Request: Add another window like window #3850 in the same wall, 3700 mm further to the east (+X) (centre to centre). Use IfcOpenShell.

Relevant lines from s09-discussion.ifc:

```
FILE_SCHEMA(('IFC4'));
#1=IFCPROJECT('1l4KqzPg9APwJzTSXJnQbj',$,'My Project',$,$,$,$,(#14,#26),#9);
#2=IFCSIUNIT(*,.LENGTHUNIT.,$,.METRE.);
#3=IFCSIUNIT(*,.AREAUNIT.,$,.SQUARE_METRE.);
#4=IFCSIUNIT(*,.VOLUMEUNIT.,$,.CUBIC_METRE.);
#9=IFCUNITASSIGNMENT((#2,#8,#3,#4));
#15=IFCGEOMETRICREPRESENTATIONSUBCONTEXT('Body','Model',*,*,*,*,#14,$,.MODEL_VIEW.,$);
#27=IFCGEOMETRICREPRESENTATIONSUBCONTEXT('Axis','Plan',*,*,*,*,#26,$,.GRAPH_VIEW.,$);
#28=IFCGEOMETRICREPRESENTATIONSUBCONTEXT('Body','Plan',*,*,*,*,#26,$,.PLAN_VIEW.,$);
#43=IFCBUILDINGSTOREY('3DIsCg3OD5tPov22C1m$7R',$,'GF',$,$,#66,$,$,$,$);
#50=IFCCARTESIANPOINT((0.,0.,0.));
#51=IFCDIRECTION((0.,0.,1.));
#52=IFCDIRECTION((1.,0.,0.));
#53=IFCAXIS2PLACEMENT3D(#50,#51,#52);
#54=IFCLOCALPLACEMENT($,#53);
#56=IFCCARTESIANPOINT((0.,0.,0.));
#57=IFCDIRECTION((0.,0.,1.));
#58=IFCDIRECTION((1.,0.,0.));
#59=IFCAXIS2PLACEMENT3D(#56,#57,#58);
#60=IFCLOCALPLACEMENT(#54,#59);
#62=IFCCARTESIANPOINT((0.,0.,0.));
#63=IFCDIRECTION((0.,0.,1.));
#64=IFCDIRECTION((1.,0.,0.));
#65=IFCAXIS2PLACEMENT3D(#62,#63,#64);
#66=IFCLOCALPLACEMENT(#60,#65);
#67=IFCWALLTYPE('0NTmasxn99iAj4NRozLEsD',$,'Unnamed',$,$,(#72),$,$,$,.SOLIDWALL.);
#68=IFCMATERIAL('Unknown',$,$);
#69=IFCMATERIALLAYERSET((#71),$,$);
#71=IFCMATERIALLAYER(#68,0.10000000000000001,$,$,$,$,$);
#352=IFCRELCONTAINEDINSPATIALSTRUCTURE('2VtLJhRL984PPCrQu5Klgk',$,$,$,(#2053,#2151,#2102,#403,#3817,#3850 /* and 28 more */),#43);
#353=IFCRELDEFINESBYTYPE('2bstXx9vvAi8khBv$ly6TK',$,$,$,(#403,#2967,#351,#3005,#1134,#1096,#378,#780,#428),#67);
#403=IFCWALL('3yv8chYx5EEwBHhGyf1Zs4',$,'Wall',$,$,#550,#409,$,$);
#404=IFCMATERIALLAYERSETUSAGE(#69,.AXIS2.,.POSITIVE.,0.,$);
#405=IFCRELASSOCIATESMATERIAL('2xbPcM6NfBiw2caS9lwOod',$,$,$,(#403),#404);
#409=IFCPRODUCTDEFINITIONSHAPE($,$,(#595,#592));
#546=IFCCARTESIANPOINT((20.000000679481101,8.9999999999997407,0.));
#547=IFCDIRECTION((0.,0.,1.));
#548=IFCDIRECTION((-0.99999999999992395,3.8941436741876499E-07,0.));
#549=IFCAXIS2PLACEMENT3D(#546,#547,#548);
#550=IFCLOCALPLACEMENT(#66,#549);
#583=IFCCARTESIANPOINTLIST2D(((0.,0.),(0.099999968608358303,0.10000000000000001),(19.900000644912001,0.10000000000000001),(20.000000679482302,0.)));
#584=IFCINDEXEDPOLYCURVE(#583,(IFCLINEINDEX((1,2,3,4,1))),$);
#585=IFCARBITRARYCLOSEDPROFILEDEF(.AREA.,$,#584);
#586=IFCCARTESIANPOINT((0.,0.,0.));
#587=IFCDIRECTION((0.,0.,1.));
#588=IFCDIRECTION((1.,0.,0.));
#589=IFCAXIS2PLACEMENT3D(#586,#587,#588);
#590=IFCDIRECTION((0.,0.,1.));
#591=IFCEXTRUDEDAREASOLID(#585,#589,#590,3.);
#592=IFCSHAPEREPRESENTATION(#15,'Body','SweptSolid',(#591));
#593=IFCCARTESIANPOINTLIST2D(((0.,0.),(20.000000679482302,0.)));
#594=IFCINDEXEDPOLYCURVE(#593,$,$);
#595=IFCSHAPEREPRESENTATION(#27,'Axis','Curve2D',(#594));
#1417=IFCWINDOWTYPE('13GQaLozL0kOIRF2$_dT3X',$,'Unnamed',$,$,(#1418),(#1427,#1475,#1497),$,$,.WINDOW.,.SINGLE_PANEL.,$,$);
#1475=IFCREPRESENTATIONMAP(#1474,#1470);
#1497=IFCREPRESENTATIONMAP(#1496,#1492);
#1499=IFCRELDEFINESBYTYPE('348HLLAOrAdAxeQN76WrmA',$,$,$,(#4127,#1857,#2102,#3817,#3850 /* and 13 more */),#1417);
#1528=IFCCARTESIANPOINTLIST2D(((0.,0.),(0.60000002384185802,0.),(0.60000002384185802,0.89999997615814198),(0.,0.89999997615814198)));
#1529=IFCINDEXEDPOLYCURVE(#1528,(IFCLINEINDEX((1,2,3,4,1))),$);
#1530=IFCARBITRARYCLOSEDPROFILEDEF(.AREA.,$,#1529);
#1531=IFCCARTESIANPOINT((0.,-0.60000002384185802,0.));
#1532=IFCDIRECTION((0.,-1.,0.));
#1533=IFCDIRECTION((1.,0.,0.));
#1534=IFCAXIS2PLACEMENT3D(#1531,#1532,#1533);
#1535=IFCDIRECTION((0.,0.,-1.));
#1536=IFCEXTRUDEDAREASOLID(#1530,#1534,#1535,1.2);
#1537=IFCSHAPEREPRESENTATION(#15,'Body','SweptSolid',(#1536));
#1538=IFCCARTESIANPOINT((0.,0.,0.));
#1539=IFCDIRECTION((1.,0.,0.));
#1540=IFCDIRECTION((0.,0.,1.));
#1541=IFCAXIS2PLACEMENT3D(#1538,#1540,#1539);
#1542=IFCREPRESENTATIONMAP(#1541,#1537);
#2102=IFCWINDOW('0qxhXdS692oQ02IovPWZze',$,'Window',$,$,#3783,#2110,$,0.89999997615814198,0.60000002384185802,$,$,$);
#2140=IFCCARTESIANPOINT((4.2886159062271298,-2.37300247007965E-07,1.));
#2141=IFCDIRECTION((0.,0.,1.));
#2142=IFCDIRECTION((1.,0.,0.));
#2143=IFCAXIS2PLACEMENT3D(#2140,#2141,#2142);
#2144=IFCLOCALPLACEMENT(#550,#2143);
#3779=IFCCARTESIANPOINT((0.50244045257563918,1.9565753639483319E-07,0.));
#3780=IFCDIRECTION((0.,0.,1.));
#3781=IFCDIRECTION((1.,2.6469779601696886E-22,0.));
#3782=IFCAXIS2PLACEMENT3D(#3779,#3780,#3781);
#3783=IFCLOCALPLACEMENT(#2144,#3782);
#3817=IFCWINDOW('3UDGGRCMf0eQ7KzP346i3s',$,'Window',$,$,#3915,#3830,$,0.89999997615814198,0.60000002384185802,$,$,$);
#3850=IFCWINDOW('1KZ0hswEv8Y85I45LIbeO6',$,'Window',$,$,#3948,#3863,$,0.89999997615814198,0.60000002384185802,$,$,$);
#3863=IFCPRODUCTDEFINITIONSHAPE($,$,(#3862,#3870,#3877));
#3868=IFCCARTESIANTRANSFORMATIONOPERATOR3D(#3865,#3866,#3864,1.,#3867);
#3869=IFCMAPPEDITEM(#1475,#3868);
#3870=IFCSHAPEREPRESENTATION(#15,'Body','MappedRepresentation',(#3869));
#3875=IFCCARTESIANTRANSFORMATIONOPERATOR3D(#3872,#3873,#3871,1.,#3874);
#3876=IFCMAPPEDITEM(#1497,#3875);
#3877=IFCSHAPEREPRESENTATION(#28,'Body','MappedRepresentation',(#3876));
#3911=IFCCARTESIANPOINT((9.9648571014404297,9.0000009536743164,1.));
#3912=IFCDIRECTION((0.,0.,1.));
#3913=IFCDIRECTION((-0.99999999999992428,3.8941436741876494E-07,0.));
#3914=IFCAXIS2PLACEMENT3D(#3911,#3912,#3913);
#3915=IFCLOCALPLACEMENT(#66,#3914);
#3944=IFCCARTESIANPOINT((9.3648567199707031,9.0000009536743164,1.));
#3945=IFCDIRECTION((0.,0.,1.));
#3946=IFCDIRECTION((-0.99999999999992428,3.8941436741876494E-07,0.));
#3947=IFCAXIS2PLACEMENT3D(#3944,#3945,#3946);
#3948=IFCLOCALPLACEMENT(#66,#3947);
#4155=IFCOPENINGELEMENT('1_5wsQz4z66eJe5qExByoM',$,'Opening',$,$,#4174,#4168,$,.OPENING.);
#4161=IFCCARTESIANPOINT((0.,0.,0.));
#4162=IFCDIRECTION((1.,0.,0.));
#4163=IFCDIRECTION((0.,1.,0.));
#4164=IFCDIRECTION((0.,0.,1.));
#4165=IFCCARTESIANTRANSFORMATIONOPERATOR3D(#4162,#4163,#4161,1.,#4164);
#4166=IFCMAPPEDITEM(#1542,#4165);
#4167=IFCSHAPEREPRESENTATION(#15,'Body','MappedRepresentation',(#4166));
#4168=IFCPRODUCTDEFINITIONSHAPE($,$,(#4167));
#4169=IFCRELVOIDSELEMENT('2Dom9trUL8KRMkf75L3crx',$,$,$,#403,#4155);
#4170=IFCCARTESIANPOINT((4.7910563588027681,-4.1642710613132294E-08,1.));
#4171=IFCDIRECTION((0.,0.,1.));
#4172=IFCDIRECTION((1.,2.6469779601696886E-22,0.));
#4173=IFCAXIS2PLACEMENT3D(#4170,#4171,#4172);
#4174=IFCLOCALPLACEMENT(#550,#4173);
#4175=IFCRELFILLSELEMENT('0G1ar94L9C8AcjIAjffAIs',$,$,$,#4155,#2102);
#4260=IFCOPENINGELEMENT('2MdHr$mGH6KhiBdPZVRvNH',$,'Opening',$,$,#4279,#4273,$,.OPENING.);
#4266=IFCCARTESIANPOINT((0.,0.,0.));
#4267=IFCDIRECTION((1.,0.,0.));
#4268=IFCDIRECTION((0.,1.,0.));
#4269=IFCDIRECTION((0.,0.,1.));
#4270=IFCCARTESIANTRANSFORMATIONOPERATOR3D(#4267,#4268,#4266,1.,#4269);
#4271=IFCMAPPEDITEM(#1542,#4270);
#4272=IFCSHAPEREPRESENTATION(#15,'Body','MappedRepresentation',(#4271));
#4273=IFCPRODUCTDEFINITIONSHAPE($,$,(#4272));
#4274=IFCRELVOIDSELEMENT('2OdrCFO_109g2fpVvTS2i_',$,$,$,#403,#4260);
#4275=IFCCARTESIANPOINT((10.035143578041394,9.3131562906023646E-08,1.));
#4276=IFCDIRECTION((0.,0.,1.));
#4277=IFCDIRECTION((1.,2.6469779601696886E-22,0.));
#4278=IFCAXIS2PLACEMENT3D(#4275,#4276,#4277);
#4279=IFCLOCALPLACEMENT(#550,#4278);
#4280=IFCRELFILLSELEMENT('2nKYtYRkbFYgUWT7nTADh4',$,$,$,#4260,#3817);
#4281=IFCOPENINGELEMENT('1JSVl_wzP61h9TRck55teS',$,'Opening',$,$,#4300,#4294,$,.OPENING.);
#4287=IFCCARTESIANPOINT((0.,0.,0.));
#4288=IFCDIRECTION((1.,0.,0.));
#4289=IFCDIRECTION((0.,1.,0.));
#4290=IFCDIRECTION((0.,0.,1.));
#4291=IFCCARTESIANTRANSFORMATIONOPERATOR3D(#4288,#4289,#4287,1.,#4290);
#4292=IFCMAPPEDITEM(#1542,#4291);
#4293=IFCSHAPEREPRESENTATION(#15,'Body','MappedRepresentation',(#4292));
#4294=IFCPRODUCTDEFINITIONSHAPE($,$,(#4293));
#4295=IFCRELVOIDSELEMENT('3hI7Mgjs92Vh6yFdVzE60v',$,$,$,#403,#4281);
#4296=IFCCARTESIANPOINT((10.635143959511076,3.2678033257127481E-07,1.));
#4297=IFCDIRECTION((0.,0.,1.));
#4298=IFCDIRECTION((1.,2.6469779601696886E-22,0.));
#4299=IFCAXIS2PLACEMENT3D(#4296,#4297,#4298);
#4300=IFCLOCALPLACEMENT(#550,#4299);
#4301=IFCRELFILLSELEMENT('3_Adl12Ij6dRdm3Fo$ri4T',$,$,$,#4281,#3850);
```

```python
import ifcopenshell
import ifcopenshell.api.feature
import ifcopenshell.api.geometry
import ifcopenshell.api.root
import ifcopenshell.geom
import ifcopenshell.util.element
import ifcopenshell.util.placement
import ifcopenshell.util.shape

model = ifcopenshell.open("s09-discussion.ifc")
settings = ifcopenshell.geom.settings()


def volume(element):
    """Net volume in cubic metres, openings subtracted."""
    shape = ifcopenshell.geom.create_shape(settings, element)
    return ifcopenshell.util.shape.get_volume(shape.geometry)


window = model.by_id(3850)
opening = window.FillsVoids[0].RelatingOpeningElement
wall = opening.VoidsElements[0].RelatingBuildingElement
before = volume(wall)
shift = ifcopenshell.util.placement.get_local_placement(wall.ObjectPlacement)[:3, 0] * -3.7

# copy_class copies the void relationship, type, container and properties, but no geometry.
new_opening = ifcopenshell.api.root.copy_class(model, product=opening)
new_opening.Representation = ifcopenshell.util.element.copy_deep(
    model, opening.Representation, exclude=["IfcGeometricRepresentationContext", "IfcRepresentationMap"]
)
new_window = ifcopenshell.api.root.copy_class(model, product=window)
new_window.Representation = ifcopenshell.util.element.copy_deep(
    model, window.Representation, exclude=["IfcGeometricRepresentationContext", "IfcRepresentationMap"]
)
ifcopenshell.api.feature.add_filling(model, opening=new_opening, element=new_window)

for old, new in ((opening, new_opening), (window, new_window)):
    matrix = ifcopenshell.util.placement.get_local_placement(old.ObjectPlacement)
    matrix[:3, 3] += shift
    ifcopenshell.api.geometry.edit_object_placement(model, product=new, matrix=matrix, is_si=False)

after = volume(wall)

print(f"wall volume {before:.3f} -> {after:.3f} m3")

model.write("s09-discussion_edited.ifc")
```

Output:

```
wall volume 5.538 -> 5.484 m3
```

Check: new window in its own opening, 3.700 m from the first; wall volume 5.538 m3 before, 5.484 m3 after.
